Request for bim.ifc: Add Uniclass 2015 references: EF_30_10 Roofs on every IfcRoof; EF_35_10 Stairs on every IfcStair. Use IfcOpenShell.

First a look at what the model holds.

```python
import ifcopenshell

model = ifcopenshell.open("bim.ifc")
print(model.schema)
print("classifications:", [c.Name for c in model.by_type("IfcClassification")])
for ifc_class in ("IfcDoor", "IfcRoof", "IfcStair", "IfcWall", "IfcWindow"):
    print(ifc_class, len(model.by_type(ifc_class)))
```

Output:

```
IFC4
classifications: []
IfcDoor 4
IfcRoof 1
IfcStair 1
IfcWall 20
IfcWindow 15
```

```python
import ifcopenshell
import ifcopenshell.api.classification

model = ifcopenshell.open("bim.ifc")

system = ifcopenshell.api.classification.add_classification(model, classification="Uniclass 2015")

codes = {
    "IfcRoof": ("EF_30_10", "Roofs"),
    "IfcStair": ("EF_35_10", "Stairs"),
}
for ifc_class, (code, name) in codes.items():
    products = model.by_type(ifc_class)
    ifcopenshell.api.classification.add_reference(
        model, products=products, classification=system, identification=code, name=name
    )
    print(code, len(products))

model.write("bim_updated.ifc")
```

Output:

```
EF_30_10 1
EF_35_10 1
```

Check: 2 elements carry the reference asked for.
